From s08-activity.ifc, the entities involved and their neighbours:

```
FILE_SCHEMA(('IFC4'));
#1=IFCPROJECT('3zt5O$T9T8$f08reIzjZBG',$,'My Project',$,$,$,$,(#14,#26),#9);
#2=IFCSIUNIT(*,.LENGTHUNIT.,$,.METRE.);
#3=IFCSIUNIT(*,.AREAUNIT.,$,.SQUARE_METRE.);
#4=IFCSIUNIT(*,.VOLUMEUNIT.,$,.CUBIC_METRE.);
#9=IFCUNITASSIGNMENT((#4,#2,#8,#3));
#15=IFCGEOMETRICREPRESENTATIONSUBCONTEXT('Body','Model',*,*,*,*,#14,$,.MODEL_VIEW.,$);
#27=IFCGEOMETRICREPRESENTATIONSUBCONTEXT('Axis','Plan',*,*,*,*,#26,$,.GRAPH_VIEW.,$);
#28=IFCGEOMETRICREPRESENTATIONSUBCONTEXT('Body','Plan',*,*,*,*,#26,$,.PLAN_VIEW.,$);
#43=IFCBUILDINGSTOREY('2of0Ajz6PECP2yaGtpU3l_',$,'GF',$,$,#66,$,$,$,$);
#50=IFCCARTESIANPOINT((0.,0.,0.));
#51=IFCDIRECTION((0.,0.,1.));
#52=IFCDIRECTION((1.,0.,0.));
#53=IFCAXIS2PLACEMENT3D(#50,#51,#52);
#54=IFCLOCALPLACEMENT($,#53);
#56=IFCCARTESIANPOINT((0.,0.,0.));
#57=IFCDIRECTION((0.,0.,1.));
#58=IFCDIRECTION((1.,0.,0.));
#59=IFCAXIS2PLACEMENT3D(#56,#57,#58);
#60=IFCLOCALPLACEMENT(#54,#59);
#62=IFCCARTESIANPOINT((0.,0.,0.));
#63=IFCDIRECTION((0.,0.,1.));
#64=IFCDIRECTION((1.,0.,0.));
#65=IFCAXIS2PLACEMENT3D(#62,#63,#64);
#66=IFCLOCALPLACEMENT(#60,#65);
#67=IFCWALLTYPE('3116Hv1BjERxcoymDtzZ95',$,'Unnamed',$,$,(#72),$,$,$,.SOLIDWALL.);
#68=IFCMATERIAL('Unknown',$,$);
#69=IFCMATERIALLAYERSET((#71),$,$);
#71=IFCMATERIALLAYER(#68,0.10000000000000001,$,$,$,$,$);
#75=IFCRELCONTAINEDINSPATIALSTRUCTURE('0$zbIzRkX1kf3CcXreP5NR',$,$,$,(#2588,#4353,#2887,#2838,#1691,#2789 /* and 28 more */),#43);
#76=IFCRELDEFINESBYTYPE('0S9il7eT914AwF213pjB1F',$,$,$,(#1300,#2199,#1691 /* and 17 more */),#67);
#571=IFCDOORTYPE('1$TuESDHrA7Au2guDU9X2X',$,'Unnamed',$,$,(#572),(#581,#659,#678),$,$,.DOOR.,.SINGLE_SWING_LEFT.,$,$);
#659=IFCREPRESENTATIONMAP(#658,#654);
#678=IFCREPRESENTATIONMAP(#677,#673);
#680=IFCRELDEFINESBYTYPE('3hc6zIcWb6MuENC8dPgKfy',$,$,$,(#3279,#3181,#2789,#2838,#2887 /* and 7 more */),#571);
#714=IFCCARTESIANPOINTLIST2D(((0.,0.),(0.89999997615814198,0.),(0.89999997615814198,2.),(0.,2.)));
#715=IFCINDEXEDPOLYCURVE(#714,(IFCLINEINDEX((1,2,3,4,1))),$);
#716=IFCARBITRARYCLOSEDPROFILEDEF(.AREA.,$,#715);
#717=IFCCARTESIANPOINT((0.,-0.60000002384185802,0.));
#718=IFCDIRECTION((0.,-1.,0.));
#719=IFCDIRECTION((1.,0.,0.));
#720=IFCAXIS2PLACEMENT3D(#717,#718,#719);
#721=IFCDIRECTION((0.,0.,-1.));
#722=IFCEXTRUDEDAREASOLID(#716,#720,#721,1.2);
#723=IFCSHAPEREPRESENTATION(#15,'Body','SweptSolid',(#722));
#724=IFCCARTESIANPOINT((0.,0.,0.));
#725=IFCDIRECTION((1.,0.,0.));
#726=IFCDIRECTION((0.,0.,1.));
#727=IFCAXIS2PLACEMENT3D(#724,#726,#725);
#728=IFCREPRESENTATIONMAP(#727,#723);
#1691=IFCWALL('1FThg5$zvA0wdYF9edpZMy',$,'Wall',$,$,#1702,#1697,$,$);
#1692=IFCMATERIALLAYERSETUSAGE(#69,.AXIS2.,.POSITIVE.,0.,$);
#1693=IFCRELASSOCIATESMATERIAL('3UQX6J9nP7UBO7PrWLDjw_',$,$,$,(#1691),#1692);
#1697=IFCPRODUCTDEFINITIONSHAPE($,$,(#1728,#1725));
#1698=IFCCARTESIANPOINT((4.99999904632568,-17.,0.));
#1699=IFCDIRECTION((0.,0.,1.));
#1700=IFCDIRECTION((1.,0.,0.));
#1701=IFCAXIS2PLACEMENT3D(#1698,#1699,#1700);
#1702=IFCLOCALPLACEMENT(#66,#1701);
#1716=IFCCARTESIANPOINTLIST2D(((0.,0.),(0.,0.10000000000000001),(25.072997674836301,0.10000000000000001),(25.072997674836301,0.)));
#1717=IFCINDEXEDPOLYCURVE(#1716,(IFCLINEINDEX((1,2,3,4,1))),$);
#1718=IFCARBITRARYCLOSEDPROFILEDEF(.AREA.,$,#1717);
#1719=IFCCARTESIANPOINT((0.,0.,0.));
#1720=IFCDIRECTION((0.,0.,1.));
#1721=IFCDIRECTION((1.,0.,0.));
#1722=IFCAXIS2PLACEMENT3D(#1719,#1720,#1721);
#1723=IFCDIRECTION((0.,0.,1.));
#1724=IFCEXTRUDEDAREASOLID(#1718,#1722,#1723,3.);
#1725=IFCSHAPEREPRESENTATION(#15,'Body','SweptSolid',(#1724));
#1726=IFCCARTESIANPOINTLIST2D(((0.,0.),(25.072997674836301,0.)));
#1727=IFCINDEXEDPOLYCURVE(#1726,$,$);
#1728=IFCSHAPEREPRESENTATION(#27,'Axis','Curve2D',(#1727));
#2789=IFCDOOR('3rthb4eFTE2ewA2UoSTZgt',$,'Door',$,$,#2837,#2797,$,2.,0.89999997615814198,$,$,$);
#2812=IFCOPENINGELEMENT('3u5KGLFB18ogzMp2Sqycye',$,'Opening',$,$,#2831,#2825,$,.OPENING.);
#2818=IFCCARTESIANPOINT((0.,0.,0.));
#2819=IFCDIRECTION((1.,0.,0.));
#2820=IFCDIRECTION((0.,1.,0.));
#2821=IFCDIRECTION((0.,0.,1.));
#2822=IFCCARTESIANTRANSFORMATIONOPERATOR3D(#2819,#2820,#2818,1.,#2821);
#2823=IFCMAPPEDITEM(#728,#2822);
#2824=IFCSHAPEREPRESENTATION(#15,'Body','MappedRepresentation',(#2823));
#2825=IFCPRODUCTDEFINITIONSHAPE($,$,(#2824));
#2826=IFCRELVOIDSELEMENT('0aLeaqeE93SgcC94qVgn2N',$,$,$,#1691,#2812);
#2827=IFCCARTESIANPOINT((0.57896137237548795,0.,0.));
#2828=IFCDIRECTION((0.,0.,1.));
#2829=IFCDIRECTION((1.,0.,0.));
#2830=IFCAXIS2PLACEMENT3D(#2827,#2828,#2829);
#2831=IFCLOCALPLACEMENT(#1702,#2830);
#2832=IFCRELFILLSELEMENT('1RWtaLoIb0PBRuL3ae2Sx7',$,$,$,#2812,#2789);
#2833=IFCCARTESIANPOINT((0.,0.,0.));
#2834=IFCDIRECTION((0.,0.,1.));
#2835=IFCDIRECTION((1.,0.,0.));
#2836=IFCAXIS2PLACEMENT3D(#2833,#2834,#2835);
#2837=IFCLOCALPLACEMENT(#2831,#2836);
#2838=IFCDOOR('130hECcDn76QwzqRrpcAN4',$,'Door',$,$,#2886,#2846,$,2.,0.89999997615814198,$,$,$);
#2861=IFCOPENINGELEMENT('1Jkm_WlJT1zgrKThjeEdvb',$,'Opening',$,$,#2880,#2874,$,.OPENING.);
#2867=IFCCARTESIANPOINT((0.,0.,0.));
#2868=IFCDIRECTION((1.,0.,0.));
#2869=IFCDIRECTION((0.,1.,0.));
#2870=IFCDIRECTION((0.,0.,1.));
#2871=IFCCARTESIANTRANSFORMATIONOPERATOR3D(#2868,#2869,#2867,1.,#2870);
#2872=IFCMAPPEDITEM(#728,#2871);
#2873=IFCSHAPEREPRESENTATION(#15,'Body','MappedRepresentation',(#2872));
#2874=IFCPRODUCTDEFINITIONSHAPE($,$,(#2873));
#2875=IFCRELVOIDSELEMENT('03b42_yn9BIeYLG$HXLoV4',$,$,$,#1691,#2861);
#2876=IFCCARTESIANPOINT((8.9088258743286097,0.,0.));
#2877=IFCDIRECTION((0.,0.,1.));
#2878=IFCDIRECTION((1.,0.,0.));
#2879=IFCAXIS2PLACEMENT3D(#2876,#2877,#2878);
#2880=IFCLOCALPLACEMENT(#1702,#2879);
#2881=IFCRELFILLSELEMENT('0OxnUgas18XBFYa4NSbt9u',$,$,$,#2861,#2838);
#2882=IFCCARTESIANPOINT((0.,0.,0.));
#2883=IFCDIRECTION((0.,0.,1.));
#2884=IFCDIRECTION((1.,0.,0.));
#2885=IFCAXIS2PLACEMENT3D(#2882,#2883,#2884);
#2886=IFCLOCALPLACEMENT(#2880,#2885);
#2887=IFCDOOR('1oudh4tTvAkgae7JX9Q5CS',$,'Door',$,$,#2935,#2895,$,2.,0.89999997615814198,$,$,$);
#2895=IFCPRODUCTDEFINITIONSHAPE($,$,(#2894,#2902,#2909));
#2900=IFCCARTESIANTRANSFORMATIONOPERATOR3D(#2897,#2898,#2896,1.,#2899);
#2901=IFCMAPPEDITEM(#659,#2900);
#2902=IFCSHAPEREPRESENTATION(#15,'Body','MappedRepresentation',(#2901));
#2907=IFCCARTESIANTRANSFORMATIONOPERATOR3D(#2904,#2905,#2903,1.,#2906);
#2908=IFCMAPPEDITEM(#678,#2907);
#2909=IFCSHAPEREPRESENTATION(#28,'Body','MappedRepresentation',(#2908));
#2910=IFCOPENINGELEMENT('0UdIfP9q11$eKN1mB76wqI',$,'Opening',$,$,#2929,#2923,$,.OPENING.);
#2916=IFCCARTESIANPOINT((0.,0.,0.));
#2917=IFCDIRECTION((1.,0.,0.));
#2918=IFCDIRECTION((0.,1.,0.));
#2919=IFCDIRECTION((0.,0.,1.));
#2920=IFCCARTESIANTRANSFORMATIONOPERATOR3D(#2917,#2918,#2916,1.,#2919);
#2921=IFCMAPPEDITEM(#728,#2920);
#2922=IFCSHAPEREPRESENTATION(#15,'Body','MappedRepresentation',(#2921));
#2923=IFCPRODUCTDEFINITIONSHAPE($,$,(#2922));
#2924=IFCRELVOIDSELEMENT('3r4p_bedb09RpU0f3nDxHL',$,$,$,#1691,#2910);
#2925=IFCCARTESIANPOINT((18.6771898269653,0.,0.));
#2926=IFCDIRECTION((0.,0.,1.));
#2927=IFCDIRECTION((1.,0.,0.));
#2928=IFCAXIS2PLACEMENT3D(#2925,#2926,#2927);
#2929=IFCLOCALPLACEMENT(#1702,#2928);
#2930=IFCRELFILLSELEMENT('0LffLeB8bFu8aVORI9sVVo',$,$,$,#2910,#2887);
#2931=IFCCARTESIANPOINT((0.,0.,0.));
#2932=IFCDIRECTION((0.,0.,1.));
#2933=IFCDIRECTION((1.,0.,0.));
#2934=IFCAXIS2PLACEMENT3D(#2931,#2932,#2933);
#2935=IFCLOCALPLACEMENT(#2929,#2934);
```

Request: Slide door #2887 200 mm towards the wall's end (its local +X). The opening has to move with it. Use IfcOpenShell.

```python
import ifcopenshell
import ifcopenshell.api.geometry
import ifcopenshell.util.placement
import ifcopenshell.util.unit

model = ifcopenshell.open("s08-activity.ifc")
unit_scale = ifcopenshell.util.unit.calculate_unit_scale(model)

door = model.by_id(2887)
opening = door.FillsVoids[0].RelatingOpeningElement
wall = opening.VoidsElements[0].RelatingBuildingElement

wall_matrix = ifcopenshell.util.placement.get_local_placement(wall.ObjectPlacement)
shift = wall_matrix[:3, 0] * 0.2 / unit_scale
before = ifcopenshell.util.placement.get_local_placement(door.ObjectPlacement)[:3, 3].copy()

# The door is placed relative to its opening, so it follows when the opening moves.
matrix = ifcopenshell.util.placement.get_local_placement(opening.ObjectPlacement)
matrix[:3, 3] += shift
ifcopenshell.api.geometry.edit_object_placement(
    model, product=opening, matrix=matrix, is_si=False, should_transform_children=True
)

after = ifcopenshell.util.placement.get_local_placement(door.ObjectPlacement)[:3, 3]
print("door moved by", (after - before).round(3) + 0.0)

model.write("s08-activity_edited.ifc")
```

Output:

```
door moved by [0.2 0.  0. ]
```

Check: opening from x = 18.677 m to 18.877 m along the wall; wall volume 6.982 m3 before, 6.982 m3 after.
